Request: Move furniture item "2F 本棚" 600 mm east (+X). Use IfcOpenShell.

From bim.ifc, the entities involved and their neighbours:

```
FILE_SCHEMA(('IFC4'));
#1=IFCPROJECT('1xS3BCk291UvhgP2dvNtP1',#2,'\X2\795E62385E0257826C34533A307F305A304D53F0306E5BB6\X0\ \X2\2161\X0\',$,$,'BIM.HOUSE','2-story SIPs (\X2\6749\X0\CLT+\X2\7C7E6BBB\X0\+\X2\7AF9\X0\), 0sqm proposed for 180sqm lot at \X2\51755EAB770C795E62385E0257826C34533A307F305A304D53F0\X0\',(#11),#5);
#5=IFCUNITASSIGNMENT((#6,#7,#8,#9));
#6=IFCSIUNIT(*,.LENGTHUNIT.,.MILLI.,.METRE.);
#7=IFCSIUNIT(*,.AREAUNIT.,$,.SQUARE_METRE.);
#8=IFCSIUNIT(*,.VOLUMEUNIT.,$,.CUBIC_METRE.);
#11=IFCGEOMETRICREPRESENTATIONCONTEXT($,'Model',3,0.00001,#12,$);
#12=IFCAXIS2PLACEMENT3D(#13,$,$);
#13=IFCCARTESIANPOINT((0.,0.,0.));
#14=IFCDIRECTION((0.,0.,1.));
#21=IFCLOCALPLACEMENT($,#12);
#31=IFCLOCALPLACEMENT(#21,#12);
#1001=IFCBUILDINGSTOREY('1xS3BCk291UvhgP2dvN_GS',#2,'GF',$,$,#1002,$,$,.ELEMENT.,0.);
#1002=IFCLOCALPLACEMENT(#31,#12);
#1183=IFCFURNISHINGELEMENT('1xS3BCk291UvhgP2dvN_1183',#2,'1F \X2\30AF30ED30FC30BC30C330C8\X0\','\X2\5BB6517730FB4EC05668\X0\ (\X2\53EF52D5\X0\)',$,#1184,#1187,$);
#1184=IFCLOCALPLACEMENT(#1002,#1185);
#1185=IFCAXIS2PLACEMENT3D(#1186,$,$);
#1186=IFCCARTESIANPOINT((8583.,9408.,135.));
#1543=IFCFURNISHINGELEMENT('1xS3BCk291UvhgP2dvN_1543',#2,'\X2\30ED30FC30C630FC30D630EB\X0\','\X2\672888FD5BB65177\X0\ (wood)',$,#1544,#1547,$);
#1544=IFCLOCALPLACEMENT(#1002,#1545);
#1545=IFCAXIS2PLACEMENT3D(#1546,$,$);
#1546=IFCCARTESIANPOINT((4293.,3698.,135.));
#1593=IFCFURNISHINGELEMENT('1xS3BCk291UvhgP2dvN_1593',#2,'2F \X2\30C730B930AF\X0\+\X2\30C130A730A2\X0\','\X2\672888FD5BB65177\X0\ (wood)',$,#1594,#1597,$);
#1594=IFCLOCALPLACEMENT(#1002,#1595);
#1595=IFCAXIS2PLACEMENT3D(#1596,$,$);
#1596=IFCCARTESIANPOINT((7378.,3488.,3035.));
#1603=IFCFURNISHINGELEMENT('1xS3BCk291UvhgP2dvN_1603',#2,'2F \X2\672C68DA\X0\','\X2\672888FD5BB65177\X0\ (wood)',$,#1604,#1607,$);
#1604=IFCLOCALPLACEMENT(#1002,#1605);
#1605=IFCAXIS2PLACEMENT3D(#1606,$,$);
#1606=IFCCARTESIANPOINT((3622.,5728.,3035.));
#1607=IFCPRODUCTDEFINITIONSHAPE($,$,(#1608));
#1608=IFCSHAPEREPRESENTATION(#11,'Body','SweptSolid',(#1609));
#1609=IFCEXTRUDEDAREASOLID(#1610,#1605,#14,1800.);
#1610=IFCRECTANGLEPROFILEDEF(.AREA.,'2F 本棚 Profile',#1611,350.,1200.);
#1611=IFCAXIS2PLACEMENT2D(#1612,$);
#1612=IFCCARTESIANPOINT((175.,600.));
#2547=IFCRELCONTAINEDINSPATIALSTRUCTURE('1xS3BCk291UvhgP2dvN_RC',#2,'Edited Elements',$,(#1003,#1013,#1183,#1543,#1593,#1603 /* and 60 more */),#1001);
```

```python
import ifcopenshell
import ifcopenshell.api.geometry
import ifcopenshell.util.placement

model = ifcopenshell.open("bim.ifc")

item = model.by_id(1603)
matrix = ifcopenshell.util.placement.get_local_placement(item.ObjectPlacement)
matrix[0, 3] += 600.0
ifcopenshell.api.geometry.edit_object_placement(model, product=item, matrix=matrix, is_si=False)

print(ifcopenshell.util.placement.get_local_placement(item.ObjectPlacement).round(3) + 0.0)

model.write("bim-out.ifc")
```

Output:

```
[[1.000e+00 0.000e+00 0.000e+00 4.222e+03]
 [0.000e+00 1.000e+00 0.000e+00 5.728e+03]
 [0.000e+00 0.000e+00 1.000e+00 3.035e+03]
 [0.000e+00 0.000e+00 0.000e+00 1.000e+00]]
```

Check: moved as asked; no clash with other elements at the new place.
